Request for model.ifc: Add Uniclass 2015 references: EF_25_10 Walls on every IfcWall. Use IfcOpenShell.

First a look at what the model holds.

```python
import ifcopenshell

model = ifcopenshell.open("model.ifc")
print(model.schema)
print("classifications:", [c.Name for c in model.by_type("IfcClassification")])
for ifc_class in ("IfcDoor", "IfcRoof", "IfcStair", "IfcWall", "IfcWindow"):
    print(ifc_class, len(model.by_type(ifc_class)))
```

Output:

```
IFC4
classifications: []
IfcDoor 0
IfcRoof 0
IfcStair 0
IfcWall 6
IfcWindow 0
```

```python
import ifcopenshell
import ifcopenshell.api.classification

model = ifcopenshell.open("model.ifc")

system = ifcopenshell.api.classification.add_classification(model, classification="Uniclass 2015")

codes = {
    "IfcWall": ("EF_25_10", "Walls"),
}
for ifc_class, (code, name) in codes.items():
    products = model.by_type(ifc_class)
    ifcopenshell.api.classification.add_reference(
        model, products=products, classification=system, identification=code, name=name
    )
    print(code, len(products))

model.write("model_edited.ifc")
```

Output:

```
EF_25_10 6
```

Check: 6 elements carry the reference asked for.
